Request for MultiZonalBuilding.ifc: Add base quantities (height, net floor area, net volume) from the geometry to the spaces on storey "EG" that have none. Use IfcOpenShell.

First a look at what the model holds.

```python
import ifcopenshell
import ifcopenshell.util.element
import ifcopenshell.util.unit

model = ifcopenshell.open("MultiZonalBuilding.ifc")
print(model.schema)
for unit_type in ("LENGTHUNIT", "AREAUNIT", "VOLUMEUNIT"):
    print(unit_type, ifcopenshell.util.unit.calculate_unit_scale(model, unit_type))
storey = next(s for s in model.by_type("IfcBuildingStorey") if s.Name == "EG")
spaces = [e for e in ifcopenshell.util.element.get_decomposition(storey) if e.is_a("IfcSpace")]
for e in sorted(spaces, key=lambda e: e.id()):
    print(e.id(), e.is_a(), e.Name, list(ifcopenshell.util.element.get_psets(e, qtos_only=True)), sep=" | ")
```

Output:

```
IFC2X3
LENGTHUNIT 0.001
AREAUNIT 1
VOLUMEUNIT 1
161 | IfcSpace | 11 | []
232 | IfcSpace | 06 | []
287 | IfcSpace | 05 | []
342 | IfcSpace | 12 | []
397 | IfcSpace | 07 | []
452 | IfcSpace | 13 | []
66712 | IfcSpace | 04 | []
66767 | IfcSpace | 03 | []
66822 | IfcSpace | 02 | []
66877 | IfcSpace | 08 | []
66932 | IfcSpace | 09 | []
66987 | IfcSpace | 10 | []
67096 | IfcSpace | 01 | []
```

```python
import ifcopenshell
import ifcopenshell.api.pset
import ifcopenshell.geom
import ifcopenshell.util.element
import ifcopenshell.util.shape
import ifcopenshell.util.unit

model = ifcopenshell.open("MultiZonalBuilding.ifc")
unit_scale = ifcopenshell.util.unit.calculate_unit_scale(model)
area_scale = ifcopenshell.util.unit.calculate_unit_scale(model, "AREAUNIT")
volume_scale = ifcopenshell.util.unit.calculate_unit_scale(model, "VOLUMEUNIT")
settings = ifcopenshell.geom.settings()

storey = next(s for s in model.by_type("IfcBuildingStorey") if s.Name == "EG")
spaces = [e for e in ifcopenshell.util.element.get_decomposition(storey) if e.is_a("IfcSpace")]

for e in sorted(spaces, key=lambda e: e.id()):
    if ifcopenshell.util.element.get_psets(e, qtos_only=True, should_inherit=False):
        continue
    # Geometry comes back in metres, in the element's own axes.
    shape = ifcopenshell.geom.create_shape(settings, e)
    values = {
        "Height": ifcopenshell.util.shape.get_z(shape.geometry) / unit_scale,
        "NetFloorArea": ifcopenshell.util.shape.get_footprint_area(shape.geometry) / area_scale,
        "NetVolume": ifcopenshell.util.shape.get_volume(shape.geometry) / volume_scale,
    }
    qto = ifcopenshell.api.pset.add_qto(model, product=e, name="BaseQuantities")
    ifcopenshell.api.pset.edit_qto(model, qto=qto, properties=values)
    print(e.id(), {k: round(v, 3) for k, v in values.items()})

model.write("MultiZonalBuilding_v2.ifc")
```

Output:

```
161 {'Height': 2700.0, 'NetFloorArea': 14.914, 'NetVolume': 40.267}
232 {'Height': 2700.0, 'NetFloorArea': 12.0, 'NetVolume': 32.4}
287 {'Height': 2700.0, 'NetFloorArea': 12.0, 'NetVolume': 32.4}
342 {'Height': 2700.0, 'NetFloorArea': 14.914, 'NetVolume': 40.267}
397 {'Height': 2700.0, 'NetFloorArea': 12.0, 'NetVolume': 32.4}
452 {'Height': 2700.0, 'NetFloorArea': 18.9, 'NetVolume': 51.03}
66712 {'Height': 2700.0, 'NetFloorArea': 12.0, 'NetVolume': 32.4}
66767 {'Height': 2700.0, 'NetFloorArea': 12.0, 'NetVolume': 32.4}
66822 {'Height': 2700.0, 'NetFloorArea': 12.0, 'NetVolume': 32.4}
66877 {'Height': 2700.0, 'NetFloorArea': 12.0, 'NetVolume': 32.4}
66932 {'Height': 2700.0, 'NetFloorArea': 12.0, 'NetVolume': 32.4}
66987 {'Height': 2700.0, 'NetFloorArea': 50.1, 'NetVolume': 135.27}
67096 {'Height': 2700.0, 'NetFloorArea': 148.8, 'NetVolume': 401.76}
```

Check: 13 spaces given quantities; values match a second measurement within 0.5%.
